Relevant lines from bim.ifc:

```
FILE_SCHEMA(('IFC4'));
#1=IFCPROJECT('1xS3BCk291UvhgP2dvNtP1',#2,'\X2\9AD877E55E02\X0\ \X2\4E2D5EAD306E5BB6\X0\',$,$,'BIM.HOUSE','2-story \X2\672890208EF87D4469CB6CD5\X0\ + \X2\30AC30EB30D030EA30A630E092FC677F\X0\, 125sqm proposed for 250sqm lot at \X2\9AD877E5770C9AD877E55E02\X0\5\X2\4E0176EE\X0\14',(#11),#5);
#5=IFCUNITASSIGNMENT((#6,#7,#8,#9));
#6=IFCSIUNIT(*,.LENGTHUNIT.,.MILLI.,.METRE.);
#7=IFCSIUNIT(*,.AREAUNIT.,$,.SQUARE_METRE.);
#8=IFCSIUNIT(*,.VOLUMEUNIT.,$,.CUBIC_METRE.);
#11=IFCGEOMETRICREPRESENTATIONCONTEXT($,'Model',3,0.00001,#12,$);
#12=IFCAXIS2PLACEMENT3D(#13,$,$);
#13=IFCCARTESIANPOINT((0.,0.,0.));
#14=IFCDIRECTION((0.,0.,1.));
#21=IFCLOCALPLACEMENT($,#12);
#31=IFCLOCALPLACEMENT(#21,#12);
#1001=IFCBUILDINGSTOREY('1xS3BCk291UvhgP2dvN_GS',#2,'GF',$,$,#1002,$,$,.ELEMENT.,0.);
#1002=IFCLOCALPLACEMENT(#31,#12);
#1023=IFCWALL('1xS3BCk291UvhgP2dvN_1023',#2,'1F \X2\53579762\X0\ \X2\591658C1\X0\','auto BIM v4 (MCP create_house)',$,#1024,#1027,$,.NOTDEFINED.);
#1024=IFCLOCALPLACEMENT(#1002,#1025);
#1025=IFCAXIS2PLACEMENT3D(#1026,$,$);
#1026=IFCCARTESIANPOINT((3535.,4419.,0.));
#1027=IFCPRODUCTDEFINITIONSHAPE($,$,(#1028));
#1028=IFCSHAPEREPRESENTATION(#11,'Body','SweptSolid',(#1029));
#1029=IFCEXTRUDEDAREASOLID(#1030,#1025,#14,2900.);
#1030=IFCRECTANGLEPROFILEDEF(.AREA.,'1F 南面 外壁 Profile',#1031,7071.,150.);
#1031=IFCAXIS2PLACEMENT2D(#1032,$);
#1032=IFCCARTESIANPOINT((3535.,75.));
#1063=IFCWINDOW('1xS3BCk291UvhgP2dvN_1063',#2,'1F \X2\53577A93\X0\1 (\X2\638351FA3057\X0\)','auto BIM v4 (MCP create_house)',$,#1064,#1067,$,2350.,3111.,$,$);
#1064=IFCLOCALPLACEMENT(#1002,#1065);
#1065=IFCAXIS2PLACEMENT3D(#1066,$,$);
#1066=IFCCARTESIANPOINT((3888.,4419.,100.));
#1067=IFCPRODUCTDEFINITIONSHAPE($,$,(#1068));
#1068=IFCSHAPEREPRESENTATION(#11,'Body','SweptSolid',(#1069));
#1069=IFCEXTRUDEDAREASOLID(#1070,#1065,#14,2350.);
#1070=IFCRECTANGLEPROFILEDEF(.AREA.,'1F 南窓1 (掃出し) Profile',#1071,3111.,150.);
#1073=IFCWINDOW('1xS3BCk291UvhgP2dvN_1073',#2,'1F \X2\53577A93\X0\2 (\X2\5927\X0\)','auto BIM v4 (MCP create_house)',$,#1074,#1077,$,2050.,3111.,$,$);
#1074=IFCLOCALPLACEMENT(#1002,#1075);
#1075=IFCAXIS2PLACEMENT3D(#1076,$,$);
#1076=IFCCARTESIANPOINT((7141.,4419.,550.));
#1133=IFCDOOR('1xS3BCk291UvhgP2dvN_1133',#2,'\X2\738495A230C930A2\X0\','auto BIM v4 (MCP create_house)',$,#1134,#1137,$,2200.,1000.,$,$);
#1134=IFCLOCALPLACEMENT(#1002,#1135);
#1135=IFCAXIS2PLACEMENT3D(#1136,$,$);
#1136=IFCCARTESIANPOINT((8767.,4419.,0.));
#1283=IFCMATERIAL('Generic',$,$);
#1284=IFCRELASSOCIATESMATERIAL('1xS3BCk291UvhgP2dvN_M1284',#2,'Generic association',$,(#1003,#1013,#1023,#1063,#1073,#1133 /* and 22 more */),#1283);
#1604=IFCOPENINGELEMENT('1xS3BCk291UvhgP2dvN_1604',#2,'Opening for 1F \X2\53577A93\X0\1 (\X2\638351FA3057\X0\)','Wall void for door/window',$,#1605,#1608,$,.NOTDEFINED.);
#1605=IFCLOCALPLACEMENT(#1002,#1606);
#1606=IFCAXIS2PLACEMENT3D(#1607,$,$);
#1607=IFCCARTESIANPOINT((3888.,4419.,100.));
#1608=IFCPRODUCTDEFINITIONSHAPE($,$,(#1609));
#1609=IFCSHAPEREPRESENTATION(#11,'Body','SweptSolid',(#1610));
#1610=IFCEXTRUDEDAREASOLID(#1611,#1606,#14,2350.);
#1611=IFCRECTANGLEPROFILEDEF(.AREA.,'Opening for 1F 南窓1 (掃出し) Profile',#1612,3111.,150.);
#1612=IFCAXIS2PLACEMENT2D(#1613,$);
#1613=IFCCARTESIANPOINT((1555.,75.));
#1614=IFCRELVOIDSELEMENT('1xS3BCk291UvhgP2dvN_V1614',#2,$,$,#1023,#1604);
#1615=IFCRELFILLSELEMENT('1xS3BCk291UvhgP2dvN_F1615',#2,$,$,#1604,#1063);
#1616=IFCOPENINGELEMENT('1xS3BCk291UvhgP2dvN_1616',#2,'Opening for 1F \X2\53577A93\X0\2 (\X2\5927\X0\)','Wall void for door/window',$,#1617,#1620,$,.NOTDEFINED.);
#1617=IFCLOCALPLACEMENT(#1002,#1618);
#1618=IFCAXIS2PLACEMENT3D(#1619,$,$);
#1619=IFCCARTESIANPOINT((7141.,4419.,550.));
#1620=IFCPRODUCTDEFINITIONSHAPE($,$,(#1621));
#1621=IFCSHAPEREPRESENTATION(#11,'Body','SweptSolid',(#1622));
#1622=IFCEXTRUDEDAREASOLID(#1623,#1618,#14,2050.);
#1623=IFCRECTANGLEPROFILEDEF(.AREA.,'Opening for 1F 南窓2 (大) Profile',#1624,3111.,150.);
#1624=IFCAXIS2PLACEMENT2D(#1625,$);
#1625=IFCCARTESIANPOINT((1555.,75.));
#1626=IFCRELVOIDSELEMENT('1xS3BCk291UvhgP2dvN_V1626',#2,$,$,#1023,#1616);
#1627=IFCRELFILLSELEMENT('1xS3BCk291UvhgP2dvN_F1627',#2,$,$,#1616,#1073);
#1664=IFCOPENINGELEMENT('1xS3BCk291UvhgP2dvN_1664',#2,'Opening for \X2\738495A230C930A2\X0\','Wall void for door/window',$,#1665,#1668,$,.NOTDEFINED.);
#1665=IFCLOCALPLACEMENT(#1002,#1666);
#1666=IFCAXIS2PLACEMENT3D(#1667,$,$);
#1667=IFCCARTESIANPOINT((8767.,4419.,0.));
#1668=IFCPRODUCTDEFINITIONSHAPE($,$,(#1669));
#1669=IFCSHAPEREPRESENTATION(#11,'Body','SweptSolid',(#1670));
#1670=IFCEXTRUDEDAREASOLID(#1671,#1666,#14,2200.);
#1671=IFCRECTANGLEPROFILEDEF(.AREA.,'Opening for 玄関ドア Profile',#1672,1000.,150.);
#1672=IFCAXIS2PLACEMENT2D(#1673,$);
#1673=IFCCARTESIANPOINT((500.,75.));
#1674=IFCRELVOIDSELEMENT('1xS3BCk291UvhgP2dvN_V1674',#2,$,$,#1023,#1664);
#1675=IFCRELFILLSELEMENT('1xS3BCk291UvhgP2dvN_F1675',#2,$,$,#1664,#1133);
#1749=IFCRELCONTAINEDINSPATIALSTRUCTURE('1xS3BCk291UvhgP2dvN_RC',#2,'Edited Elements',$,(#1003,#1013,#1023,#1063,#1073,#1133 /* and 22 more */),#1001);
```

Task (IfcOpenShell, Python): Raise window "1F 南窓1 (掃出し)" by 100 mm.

```python
import numpy as np
import ifcopenshell
import ifcopenshell.api.geometry
import ifcopenshell.util.placement
import ifcopenshell.util.unit

model = ifcopenshell.open("bim.ifc")
unit_scale = ifcopenshell.util.unit.calculate_unit_scale(model)

window = model.by_guid("1xS3BCk291UvhgP2dvN_1063")
opening = window.FillsVoids[0].RelatingOpeningElement
dz = 0.1 / unit_scale

shift = np.array([0.0, 0.0, dz])
# The window is not placed relative to its opening, so move both.
for product in (opening, window):
    matrix = ifcopenshell.util.placement.get_local_placement(product.ObjectPlacement)
    matrix[:3, 3] += shift
    ifcopenshell.api.geometry.edit_object_placement(model, product=product, matrix=matrix, is_si=False)

print(f"moved by {dz * unit_scale:+.3f} m")

model.write("bim-out.ifc")
```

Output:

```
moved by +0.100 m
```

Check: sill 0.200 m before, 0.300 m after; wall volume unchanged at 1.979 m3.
